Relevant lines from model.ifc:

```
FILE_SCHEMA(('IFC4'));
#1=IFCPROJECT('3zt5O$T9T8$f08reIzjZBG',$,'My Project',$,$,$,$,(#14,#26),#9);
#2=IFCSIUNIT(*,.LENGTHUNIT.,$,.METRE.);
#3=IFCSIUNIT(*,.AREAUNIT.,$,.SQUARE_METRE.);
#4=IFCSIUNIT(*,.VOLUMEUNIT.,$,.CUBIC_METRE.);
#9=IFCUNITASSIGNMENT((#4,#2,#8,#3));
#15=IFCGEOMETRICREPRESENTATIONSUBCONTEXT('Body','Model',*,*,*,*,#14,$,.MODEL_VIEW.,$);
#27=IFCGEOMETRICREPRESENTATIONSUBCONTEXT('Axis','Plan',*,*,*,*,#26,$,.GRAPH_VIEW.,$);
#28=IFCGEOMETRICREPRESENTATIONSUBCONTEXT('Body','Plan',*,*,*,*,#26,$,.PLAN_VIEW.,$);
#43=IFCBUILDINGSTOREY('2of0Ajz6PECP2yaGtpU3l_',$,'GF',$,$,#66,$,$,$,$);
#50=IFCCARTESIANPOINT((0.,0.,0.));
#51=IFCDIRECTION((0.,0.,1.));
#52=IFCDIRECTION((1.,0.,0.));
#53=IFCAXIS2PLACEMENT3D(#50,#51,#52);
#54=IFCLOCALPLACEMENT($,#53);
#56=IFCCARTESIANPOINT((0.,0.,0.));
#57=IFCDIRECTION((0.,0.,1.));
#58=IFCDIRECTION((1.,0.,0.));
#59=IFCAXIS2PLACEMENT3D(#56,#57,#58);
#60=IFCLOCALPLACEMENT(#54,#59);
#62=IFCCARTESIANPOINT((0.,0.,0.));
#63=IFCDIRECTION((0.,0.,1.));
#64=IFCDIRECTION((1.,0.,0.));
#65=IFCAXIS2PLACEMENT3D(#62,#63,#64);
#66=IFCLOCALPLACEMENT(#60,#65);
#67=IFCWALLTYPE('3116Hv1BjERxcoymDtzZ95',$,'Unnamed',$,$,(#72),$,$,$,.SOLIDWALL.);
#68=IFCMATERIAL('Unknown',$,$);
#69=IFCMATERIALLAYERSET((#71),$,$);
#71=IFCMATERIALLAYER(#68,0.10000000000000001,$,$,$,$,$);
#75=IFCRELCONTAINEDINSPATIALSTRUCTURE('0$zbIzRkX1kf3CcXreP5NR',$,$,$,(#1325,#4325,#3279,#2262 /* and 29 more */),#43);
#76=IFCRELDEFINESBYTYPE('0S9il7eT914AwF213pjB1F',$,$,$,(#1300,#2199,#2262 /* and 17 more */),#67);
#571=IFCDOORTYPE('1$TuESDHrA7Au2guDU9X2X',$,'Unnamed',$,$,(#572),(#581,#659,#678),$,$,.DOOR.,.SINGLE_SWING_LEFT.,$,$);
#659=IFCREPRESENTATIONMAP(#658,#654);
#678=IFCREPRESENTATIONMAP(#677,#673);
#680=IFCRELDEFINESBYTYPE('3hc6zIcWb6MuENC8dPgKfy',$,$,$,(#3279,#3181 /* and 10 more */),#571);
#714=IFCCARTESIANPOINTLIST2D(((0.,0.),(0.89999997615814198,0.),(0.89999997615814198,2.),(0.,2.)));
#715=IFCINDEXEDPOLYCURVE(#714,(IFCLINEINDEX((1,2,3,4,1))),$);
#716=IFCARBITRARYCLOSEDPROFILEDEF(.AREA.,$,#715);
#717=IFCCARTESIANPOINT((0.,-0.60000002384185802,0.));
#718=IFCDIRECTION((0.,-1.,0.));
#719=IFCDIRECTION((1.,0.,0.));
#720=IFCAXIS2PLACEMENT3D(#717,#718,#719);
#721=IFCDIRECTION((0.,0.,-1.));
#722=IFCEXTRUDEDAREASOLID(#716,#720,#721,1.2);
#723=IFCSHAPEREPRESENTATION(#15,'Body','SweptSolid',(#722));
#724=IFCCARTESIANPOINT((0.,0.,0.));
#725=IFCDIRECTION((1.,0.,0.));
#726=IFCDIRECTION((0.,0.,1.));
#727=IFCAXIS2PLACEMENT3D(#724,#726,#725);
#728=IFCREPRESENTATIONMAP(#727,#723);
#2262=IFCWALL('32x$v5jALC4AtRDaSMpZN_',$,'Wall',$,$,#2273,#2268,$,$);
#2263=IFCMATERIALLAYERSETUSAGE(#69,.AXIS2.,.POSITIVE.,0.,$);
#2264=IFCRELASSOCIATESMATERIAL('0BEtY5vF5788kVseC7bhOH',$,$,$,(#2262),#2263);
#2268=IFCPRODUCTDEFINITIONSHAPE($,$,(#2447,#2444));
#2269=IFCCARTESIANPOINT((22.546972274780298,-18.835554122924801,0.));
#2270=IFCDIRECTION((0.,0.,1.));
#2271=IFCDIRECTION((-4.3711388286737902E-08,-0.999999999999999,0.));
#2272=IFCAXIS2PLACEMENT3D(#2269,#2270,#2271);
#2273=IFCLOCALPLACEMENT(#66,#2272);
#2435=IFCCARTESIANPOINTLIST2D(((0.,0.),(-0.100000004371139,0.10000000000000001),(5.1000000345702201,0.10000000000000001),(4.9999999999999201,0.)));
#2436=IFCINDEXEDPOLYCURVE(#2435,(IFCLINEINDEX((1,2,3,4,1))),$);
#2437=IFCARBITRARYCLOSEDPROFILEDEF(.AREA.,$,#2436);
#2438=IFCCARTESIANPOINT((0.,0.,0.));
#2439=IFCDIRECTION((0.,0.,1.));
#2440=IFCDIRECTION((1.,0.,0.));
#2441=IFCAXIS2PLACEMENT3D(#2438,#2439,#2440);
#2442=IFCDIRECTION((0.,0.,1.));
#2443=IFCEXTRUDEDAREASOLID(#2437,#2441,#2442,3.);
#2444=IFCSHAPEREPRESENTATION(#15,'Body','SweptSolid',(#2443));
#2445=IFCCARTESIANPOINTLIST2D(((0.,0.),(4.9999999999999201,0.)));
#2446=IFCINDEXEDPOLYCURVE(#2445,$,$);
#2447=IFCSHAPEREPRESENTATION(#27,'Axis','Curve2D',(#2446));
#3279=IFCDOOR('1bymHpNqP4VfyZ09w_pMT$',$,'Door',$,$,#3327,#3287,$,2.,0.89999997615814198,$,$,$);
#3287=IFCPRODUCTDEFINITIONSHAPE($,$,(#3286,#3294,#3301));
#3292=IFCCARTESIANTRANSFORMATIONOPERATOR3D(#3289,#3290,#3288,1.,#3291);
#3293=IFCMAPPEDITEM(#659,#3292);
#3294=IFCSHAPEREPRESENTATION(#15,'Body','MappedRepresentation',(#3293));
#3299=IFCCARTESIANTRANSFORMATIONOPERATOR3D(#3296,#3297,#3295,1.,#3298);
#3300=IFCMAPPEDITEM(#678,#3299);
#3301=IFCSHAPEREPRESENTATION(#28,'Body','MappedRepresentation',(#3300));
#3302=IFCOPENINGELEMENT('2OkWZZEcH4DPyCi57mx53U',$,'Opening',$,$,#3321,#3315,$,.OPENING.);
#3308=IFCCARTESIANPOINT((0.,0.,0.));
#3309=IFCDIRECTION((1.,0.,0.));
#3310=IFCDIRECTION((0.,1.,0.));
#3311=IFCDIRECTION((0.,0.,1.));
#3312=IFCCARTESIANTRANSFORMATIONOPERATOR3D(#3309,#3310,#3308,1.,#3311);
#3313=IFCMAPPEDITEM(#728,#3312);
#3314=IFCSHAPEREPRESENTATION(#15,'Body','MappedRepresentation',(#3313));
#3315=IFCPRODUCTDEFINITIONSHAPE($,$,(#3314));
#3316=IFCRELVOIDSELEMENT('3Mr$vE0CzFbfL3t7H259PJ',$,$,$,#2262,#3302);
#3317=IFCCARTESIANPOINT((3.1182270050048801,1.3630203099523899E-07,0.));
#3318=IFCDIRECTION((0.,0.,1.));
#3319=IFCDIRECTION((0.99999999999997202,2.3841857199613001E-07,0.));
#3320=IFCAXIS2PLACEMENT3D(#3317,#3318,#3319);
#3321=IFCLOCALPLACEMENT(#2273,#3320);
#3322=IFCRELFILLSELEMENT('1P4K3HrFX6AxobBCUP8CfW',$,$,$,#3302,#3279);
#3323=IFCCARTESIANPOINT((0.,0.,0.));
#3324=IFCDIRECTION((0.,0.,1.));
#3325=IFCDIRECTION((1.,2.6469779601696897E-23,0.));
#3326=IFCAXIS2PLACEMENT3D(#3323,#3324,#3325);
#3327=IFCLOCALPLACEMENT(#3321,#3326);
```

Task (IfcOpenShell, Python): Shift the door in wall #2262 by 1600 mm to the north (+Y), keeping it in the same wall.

```python
import ifcopenshell
import ifcopenshell.api.geometry
import ifcopenshell.util.placement
import ifcopenshell.util.unit

model = ifcopenshell.open("model.ifc")
unit_scale = ifcopenshell.util.unit.calculate_unit_scale(model)

door = model.by_guid("1bymHpNqP4VfyZ09w_pMT$")
opening = door.FillsVoids[0].RelatingOpeningElement
wall = opening.VoidsElements[0].RelatingBuildingElement

wall_matrix = ifcopenshell.util.placement.get_local_placement(wall.ObjectPlacement)
shift = wall_matrix[:3, 0] * -1.6 / unit_scale
before = ifcopenshell.util.placement.get_local_placement(door.ObjectPlacement)[:3, 3].copy()

# The door is placed relative to its opening, so it follows when the opening moves.
matrix = ifcopenshell.util.placement.get_local_placement(opening.ObjectPlacement)
matrix[:3, 3] += shift
ifcopenshell.api.geometry.edit_object_placement(
    model, product=opening, matrix=matrix, is_si=False, should_transform_children=True
)

after = ifcopenshell.util.placement.get_local_placement(door.ObjectPlacement)[:3, 3]
print("door moved by", (after - before).round(3) + 0.0)

model.write("model_v2.ifc")
```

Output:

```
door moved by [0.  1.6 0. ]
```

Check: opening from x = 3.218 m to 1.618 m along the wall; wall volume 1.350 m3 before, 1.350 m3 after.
